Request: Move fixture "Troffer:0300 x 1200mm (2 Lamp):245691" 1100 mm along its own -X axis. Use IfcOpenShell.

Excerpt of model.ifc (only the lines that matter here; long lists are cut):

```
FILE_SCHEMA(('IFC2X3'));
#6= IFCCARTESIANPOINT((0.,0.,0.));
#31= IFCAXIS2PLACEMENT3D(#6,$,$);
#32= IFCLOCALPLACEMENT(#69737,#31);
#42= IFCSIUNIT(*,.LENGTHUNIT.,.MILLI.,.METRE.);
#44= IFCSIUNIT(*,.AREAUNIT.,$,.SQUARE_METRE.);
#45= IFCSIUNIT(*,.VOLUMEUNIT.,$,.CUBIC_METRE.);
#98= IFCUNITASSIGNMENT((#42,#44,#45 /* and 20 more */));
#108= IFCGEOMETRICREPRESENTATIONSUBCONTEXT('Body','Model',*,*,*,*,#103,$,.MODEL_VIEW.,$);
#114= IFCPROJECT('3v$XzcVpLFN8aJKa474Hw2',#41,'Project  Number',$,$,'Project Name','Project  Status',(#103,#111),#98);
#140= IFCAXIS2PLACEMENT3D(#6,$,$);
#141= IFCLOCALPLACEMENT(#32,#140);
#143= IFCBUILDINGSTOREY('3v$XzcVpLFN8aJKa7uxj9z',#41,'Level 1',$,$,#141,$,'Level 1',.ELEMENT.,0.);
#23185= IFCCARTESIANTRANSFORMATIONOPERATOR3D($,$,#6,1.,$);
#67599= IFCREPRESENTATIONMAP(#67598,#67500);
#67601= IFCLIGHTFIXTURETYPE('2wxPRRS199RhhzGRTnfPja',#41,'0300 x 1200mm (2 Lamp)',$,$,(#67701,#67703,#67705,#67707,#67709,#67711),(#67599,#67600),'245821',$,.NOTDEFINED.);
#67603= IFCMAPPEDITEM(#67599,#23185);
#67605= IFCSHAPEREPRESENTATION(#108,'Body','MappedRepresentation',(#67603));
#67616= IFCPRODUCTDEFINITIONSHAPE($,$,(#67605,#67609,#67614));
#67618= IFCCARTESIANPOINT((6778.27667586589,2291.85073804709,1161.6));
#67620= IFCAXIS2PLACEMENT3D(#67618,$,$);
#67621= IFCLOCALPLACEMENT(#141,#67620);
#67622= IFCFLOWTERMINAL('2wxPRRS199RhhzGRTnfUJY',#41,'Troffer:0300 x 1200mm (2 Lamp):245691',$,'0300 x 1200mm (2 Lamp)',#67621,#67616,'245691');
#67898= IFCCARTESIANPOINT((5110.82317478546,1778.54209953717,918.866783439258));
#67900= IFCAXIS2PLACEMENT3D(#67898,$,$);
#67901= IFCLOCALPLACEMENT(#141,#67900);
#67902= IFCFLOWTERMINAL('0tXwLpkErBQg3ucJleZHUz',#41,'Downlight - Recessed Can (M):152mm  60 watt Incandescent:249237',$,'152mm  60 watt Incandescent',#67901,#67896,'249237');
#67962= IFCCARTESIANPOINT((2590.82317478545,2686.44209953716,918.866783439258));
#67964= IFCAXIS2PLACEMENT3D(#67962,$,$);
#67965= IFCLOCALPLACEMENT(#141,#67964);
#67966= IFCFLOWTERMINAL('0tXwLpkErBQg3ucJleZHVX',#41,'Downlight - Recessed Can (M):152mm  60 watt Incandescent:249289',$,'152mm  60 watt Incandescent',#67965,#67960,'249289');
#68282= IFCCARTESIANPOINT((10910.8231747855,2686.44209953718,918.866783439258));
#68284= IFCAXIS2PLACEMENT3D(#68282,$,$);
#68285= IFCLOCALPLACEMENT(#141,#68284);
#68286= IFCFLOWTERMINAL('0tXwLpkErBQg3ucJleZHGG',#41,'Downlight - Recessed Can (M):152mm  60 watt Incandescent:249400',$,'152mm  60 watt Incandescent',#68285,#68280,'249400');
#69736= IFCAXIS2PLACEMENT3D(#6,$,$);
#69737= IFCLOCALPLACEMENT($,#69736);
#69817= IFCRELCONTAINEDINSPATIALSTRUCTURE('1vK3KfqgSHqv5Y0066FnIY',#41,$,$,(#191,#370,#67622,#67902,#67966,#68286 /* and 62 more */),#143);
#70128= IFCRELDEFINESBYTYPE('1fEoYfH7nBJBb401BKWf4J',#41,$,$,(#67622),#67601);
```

```python
import ifcopenshell
import ifcopenshell.api.geometry
import ifcopenshell.util.placement
import ifcopenshell.util.unit

model = ifcopenshell.open("model.ifc")
unit_scale = ifcopenshell.util.unit.calculate_unit_scale(model)

item = model.by_guid("2wxPRRS199RhhzGRTnfUJY")
matrix = ifcopenshell.util.placement.get_local_placement(item.ObjectPlacement)
matrix[:3, 3] -= matrix[:3, 0] * 1.1 / unit_scale
ifcopenshell.api.geometry.edit_object_placement(model, product=item, matrix=matrix, is_si=False)

print(ifcopenshell.util.placement.get_local_placement(item.ObjectPlacement).round(3) + 0.0)

model.write("model-out.ifc")
```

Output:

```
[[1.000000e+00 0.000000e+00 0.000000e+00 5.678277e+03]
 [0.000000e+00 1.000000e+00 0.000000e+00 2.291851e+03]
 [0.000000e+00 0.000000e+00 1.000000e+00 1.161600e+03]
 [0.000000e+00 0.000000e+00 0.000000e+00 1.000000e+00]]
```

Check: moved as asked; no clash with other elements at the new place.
